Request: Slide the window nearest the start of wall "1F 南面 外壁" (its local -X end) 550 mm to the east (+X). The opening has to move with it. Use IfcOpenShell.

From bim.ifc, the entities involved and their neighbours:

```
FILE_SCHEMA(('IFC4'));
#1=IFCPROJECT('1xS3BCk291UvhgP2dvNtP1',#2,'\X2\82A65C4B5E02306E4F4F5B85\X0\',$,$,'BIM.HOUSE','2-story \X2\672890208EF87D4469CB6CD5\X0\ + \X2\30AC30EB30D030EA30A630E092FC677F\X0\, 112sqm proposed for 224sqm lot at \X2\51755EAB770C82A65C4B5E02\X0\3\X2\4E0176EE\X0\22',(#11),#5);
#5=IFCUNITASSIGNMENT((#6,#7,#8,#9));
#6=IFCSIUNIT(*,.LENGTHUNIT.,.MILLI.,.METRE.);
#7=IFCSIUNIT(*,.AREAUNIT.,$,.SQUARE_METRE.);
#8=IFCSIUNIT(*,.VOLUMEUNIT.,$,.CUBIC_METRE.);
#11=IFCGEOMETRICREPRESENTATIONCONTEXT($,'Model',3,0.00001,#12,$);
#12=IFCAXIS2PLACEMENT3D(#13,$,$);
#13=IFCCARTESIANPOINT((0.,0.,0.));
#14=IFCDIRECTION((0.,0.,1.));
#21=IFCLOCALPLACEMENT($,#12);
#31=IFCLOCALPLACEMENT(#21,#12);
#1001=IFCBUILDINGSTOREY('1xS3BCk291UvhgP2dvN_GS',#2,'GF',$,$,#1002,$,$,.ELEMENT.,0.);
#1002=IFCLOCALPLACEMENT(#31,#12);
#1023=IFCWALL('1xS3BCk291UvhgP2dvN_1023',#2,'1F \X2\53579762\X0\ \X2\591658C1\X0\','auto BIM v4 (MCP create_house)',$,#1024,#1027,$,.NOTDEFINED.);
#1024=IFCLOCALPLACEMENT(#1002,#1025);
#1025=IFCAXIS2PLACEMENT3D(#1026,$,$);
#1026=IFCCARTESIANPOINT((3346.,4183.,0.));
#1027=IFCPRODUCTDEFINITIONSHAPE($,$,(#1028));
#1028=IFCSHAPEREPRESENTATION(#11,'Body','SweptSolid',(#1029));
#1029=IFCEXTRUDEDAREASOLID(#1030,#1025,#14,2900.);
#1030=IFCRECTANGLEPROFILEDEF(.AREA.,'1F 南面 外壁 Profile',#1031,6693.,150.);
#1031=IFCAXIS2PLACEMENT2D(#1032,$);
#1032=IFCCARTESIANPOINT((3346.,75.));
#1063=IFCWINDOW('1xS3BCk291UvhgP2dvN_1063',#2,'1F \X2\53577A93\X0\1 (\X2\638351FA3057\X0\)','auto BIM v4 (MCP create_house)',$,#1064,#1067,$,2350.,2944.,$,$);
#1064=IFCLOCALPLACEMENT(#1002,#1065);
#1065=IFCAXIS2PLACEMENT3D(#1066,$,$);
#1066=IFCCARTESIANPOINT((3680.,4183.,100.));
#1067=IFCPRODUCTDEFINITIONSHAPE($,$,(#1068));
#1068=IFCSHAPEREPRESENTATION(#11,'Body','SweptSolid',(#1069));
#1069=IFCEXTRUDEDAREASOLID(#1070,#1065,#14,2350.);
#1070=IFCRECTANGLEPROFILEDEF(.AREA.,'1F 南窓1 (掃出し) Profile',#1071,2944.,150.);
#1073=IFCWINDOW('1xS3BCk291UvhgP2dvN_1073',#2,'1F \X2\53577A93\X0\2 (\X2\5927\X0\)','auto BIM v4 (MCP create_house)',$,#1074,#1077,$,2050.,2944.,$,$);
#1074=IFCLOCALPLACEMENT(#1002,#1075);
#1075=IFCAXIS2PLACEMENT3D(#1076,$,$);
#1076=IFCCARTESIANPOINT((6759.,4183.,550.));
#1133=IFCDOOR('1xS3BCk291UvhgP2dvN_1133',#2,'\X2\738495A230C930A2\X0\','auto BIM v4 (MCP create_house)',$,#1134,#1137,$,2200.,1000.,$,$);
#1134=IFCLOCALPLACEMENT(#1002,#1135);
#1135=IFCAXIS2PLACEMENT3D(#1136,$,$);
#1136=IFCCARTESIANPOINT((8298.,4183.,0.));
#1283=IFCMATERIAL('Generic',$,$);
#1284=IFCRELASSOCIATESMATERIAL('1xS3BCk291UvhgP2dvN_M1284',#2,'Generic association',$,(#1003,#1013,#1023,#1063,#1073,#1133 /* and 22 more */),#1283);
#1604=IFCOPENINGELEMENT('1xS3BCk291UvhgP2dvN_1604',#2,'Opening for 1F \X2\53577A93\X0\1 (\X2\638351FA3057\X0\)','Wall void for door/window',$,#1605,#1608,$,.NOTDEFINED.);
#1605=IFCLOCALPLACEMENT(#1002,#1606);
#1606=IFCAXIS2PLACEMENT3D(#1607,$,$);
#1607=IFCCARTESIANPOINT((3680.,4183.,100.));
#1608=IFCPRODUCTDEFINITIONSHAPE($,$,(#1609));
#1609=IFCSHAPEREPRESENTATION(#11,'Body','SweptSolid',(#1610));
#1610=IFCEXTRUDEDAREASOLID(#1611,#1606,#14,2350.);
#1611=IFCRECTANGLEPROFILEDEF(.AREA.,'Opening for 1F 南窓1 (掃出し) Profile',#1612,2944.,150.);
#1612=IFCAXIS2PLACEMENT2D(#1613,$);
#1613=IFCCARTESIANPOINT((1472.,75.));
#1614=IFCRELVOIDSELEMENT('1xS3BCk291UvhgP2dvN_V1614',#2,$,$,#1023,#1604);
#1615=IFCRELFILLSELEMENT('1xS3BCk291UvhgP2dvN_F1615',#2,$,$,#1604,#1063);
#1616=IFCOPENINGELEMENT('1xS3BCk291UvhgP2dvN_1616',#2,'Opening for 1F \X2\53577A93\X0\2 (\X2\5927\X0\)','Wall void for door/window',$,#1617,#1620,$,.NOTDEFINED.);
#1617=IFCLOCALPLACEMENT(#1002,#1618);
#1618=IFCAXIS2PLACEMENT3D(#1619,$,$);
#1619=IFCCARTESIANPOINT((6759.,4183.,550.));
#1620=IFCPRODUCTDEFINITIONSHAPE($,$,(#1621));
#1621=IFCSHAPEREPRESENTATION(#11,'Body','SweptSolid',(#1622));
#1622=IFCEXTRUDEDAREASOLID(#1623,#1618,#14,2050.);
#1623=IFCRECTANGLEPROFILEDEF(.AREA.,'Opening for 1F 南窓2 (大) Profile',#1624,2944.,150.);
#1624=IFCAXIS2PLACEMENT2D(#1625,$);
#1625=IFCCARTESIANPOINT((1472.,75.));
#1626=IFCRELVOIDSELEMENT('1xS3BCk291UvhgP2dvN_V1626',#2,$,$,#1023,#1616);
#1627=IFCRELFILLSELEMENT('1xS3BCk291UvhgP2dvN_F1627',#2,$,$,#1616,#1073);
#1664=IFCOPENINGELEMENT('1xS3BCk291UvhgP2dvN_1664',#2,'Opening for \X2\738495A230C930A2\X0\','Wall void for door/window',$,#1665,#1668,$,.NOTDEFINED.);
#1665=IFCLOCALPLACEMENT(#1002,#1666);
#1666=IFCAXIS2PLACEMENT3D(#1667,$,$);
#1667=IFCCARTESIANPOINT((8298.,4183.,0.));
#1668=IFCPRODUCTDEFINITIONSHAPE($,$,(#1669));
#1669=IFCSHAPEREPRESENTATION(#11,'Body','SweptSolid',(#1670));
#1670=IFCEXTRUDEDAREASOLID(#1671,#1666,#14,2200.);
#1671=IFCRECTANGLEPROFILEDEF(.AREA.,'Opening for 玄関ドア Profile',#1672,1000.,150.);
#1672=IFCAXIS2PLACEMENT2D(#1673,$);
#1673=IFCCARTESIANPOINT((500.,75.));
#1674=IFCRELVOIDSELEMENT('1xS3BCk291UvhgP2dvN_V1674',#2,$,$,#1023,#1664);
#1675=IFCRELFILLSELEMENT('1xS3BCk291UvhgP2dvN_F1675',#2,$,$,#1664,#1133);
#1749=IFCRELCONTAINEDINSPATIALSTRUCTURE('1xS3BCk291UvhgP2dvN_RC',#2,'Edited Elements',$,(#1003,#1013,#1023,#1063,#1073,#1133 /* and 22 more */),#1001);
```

```python
import ifcopenshell
import ifcopenshell.api.geometry
import ifcopenshell.util.placement
import ifcopenshell.util.unit

model = ifcopenshell.open("bim.ifc")
unit_scale = ifcopenshell.util.unit.calculate_unit_scale(model)

window = model.by_guid("1xS3BCk291UvhgP2dvN_1063")
opening = window.FillsVoids[0].RelatingOpeningElement
wall = opening.VoidsElements[0].RelatingBuildingElement

wall_matrix = ifcopenshell.util.placement.get_local_placement(wall.ObjectPlacement)
shift = wall_matrix[:3, 0] * 0.55 / unit_scale
before = ifcopenshell.util.placement.get_local_placement(window.ObjectPlacement)[:3, 3].copy()

# The window is not placed relative to its opening, so move both.
for product in (opening, window):
    matrix = ifcopenshell.util.placement.get_local_placement(product.ObjectPlacement)
    matrix[:3, 3] += shift
    ifcopenshell.api.geometry.edit_object_placement(model, product=product, matrix=matrix, is_si=False)

after = ifcopenshell.util.placement.get_local_placement(window.ObjectPlacement)[:3, 3]
print("window moved by", (after - before).round(3) + 0.0)

model.write("bim_edited.ifc")
```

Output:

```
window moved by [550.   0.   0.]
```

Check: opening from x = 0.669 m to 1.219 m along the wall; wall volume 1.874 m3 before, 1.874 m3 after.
